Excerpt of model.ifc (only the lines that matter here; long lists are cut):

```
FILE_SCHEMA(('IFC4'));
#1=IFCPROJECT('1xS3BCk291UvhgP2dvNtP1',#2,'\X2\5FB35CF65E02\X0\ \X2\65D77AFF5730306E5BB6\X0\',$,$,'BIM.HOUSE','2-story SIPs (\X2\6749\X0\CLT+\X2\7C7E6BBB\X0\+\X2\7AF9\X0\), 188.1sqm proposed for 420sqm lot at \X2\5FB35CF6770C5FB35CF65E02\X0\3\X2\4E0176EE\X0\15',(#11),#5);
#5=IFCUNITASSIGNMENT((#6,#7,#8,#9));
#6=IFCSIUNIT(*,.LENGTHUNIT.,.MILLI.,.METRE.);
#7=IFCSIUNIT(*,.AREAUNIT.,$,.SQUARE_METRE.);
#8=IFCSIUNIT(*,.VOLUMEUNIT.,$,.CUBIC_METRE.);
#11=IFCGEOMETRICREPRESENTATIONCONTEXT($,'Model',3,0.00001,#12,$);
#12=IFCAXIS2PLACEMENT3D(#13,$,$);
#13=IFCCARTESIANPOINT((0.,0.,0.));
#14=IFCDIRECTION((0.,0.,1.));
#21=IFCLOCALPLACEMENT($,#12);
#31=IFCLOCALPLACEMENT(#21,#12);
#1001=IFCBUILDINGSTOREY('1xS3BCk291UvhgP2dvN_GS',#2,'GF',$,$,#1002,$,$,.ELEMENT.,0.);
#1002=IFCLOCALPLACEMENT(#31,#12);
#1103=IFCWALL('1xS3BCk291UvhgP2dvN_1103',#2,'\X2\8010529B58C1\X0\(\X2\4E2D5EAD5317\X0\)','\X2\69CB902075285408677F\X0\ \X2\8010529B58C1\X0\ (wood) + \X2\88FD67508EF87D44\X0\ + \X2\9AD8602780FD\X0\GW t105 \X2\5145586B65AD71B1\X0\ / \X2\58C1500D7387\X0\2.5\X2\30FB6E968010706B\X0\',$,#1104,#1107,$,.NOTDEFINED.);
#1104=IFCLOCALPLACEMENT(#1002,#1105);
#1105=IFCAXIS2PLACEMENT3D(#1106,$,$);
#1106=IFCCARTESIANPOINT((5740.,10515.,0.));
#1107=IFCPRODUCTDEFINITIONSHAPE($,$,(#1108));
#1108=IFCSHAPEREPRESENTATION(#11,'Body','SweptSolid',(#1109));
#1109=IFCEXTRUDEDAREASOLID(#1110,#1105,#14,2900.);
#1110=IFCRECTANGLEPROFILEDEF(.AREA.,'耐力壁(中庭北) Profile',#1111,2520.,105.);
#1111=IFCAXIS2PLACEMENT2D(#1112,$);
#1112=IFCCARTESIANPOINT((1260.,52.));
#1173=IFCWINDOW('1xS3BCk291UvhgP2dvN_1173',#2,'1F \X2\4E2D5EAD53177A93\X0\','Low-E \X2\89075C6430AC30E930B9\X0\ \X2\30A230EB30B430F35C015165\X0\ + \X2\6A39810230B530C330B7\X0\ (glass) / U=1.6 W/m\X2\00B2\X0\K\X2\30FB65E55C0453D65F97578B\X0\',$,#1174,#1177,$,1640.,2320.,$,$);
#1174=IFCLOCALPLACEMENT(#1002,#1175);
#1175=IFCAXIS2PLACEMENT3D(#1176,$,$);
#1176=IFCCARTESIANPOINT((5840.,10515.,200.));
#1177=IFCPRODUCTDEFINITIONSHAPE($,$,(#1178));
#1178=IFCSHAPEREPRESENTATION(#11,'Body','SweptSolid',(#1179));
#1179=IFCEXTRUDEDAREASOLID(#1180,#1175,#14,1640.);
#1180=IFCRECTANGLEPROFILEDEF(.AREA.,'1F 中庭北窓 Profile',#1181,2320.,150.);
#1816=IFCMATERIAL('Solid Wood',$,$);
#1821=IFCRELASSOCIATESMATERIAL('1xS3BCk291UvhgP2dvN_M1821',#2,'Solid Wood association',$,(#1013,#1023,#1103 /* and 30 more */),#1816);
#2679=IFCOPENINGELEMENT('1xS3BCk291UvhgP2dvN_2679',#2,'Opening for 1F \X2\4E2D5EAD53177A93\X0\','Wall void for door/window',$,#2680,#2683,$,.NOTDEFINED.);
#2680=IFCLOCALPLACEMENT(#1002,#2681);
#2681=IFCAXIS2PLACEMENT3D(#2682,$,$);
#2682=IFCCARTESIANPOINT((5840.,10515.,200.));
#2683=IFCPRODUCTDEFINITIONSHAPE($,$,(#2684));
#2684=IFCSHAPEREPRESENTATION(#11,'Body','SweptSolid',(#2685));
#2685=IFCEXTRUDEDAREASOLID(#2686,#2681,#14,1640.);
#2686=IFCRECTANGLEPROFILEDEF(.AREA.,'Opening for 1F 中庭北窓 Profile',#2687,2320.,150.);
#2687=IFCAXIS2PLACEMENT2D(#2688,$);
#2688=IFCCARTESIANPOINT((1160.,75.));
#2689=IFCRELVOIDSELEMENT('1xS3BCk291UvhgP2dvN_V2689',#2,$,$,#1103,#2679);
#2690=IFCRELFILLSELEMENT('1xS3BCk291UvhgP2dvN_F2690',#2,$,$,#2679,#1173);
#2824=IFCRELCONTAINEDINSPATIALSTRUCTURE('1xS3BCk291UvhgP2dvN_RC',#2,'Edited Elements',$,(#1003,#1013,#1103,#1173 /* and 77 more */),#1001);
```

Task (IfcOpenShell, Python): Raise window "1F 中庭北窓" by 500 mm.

```python
import numpy as np
import ifcopenshell
import ifcopenshell.api.geometry
import ifcopenshell.util.placement
import ifcopenshell.util.unit

model = ifcopenshell.open("model.ifc")
unit_scale = ifcopenshell.util.unit.calculate_unit_scale(model)

window = model.by_guid("1xS3BCk291UvhgP2dvN_1173")
opening = window.FillsVoids[0].RelatingOpeningElement
dz = 500.0

shift = np.array([0.0, 0.0, dz])
# The window is not placed relative to its opening, so move both.
for product in (opening, window):
    matrix = ifcopenshell.util.placement.get_local_placement(product.ObjectPlacement)
    matrix[:3, 3] += shift
    ifcopenshell.api.geometry.edit_object_placement(model, product=product, matrix=matrix, is_si=False)

print(f"moved by {dz * unit_scale:+.3f} m")

model.write("model_updated.ifc")
```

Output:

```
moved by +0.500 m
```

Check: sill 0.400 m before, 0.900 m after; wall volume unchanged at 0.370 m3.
